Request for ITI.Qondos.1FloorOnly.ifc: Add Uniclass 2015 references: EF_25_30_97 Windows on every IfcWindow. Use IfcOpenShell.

First a look at what the model holds.

```python
import ifcopenshell

model = ifcopenshell.open("ITI.Qondos.1FloorOnly.ifc")
print(model.schema)
print("classifications:", [c.Name for c in model.by_type("IfcClassification")])
for ifc_class in ("IfcDoor", "IfcRoof", "IfcStair", "IfcWall", "IfcWindow"):
    print(ifc_class, len(model.by_type(ifc_class)))
```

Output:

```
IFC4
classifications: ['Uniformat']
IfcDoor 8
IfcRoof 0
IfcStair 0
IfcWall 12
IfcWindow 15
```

```python
import ifcopenshell
import ifcopenshell.api.classification

model = ifcopenshell.open("ITI.Qondos.1FloorOnly.ifc")

system = ifcopenshell.api.classification.add_classification(model, classification="Uniclass 2015")

codes = {
    "IfcWindow": ("EF_25_30_97", "Windows"),
}
for ifc_class, (code, name) in codes.items():
    products = model.by_type(ifc_class)
    ifcopenshell.api.classification.add_reference(
        model, products=products, classification=system, identification=code, name=name
    )
    print(code, len(products))

model.write("ITI.Qondos.1FloorOnly_rev.ifc")
```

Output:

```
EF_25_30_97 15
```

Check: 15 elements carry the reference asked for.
